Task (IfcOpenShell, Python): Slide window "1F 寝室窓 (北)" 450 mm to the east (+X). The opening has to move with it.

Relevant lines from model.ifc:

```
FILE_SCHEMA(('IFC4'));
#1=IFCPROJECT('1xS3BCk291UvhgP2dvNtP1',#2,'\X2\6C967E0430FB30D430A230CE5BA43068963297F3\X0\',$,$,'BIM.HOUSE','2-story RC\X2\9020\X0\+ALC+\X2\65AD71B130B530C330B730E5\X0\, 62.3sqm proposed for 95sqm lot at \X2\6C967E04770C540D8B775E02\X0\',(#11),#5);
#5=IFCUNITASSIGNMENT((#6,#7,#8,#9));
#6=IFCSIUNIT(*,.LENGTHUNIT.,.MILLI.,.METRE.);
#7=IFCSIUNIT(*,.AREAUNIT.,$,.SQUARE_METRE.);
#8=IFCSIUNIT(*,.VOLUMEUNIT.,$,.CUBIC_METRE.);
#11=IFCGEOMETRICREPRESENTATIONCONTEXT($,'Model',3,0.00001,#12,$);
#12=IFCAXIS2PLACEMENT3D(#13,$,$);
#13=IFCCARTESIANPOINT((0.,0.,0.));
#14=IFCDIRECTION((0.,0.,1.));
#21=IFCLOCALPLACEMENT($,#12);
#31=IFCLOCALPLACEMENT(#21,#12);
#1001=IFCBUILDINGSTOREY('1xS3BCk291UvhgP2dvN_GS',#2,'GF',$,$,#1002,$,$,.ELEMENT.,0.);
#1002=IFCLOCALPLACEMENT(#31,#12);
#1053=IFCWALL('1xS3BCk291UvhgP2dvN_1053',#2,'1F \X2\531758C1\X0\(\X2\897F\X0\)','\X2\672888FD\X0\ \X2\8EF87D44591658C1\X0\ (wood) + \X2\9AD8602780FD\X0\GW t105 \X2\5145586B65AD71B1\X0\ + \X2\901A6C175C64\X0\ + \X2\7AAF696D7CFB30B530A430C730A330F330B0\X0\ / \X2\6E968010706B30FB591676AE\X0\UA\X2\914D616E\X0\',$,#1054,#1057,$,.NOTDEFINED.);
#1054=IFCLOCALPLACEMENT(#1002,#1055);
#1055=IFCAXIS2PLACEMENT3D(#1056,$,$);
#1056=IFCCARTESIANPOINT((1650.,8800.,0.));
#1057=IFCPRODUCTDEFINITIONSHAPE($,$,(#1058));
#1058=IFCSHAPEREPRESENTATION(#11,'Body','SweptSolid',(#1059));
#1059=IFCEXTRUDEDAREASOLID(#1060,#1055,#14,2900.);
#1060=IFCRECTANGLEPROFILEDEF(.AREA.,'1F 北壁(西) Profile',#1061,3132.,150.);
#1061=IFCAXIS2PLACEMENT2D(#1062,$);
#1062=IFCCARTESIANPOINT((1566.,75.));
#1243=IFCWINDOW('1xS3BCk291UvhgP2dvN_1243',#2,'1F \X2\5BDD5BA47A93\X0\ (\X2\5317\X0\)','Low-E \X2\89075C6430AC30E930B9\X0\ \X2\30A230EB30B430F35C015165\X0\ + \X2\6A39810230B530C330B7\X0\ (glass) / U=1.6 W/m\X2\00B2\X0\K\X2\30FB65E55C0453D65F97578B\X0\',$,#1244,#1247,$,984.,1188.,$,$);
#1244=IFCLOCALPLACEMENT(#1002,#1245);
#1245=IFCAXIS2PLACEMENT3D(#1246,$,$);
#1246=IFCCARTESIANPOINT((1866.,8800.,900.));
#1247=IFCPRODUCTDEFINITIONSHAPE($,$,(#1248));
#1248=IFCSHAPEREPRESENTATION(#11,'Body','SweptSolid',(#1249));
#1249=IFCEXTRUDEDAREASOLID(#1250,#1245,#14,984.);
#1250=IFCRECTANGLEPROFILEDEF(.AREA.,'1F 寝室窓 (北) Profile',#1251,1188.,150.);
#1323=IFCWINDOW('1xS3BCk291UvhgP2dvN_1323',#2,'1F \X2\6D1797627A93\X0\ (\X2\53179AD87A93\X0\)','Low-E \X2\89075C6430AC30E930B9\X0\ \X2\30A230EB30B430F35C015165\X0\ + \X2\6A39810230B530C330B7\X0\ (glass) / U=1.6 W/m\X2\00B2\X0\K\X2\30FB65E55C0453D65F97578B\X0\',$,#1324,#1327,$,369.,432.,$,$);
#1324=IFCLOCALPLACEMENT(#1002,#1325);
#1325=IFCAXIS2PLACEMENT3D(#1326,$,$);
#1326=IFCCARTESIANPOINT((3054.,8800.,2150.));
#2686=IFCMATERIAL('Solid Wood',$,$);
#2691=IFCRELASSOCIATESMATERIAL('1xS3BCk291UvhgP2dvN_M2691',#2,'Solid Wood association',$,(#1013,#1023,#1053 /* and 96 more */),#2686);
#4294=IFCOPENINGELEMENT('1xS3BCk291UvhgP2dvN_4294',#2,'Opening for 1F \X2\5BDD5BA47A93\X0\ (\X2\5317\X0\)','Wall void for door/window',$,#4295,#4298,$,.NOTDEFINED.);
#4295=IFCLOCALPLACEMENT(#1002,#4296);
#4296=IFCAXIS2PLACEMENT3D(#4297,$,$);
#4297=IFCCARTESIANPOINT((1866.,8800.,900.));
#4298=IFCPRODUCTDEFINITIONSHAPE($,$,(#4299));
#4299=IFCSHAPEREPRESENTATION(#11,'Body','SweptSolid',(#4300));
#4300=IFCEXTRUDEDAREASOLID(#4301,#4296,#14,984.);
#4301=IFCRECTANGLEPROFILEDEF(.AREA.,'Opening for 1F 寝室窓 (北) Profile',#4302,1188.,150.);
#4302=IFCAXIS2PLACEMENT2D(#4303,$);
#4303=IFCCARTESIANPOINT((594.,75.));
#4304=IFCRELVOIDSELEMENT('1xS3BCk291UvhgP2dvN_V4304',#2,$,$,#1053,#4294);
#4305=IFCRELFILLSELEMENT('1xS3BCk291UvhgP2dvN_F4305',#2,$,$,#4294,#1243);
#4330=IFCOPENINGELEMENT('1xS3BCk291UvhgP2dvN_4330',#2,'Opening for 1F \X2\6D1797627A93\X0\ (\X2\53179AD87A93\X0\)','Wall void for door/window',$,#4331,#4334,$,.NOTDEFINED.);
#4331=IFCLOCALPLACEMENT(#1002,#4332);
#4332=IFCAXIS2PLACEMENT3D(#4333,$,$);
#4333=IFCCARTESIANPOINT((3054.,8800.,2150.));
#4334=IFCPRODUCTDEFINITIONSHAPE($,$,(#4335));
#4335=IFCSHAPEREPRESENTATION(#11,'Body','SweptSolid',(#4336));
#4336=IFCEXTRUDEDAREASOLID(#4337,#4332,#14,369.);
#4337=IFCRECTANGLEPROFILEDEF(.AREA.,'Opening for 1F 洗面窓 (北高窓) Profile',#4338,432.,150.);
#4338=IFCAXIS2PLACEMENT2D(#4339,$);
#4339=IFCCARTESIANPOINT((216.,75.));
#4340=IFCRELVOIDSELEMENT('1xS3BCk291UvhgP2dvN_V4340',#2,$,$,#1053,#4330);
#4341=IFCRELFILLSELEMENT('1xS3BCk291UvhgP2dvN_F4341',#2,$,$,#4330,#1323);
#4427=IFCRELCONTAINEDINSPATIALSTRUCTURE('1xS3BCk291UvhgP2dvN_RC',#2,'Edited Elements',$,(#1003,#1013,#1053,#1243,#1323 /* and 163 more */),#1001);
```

```python
import ifcopenshell
import ifcopenshell.api.geometry
import ifcopenshell.util.placement
import ifcopenshell.util.unit

model = ifcopenshell.open("model.ifc")
unit_scale = ifcopenshell.util.unit.calculate_unit_scale(model)

window = model.by_guid("1xS3BCk291UvhgP2dvN_1243")
opening = window.FillsVoids[0].RelatingOpeningElement
wall = opening.VoidsElements[0].RelatingBuildingElement

wall_matrix = ifcopenshell.util.placement.get_local_placement(wall.ObjectPlacement)
shift = wall_matrix[:3, 0] * 0.45 / unit_scale
before = ifcopenshell.util.placement.get_local_placement(window.ObjectPlacement)[:3, 3].copy()

# The window is not placed relative to its opening, so move both.
for product in (opening, window):
    matrix = ifcopenshell.util.placement.get_local_placement(product.ObjectPlacement)
    matrix[:3, 3] += shift
    ifcopenshell.api.geometry.edit_object_placement(model, product=product, matrix=matrix, is_si=False)

after = ifcopenshell.util.placement.get_local_placement(window.ObjectPlacement)[:3, 3]
print("window moved by", (after - before).round(3) + 0.0)

model.write("model_updated.ifc")
```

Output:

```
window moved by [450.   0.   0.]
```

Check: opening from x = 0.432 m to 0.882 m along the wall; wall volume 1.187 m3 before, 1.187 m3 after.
